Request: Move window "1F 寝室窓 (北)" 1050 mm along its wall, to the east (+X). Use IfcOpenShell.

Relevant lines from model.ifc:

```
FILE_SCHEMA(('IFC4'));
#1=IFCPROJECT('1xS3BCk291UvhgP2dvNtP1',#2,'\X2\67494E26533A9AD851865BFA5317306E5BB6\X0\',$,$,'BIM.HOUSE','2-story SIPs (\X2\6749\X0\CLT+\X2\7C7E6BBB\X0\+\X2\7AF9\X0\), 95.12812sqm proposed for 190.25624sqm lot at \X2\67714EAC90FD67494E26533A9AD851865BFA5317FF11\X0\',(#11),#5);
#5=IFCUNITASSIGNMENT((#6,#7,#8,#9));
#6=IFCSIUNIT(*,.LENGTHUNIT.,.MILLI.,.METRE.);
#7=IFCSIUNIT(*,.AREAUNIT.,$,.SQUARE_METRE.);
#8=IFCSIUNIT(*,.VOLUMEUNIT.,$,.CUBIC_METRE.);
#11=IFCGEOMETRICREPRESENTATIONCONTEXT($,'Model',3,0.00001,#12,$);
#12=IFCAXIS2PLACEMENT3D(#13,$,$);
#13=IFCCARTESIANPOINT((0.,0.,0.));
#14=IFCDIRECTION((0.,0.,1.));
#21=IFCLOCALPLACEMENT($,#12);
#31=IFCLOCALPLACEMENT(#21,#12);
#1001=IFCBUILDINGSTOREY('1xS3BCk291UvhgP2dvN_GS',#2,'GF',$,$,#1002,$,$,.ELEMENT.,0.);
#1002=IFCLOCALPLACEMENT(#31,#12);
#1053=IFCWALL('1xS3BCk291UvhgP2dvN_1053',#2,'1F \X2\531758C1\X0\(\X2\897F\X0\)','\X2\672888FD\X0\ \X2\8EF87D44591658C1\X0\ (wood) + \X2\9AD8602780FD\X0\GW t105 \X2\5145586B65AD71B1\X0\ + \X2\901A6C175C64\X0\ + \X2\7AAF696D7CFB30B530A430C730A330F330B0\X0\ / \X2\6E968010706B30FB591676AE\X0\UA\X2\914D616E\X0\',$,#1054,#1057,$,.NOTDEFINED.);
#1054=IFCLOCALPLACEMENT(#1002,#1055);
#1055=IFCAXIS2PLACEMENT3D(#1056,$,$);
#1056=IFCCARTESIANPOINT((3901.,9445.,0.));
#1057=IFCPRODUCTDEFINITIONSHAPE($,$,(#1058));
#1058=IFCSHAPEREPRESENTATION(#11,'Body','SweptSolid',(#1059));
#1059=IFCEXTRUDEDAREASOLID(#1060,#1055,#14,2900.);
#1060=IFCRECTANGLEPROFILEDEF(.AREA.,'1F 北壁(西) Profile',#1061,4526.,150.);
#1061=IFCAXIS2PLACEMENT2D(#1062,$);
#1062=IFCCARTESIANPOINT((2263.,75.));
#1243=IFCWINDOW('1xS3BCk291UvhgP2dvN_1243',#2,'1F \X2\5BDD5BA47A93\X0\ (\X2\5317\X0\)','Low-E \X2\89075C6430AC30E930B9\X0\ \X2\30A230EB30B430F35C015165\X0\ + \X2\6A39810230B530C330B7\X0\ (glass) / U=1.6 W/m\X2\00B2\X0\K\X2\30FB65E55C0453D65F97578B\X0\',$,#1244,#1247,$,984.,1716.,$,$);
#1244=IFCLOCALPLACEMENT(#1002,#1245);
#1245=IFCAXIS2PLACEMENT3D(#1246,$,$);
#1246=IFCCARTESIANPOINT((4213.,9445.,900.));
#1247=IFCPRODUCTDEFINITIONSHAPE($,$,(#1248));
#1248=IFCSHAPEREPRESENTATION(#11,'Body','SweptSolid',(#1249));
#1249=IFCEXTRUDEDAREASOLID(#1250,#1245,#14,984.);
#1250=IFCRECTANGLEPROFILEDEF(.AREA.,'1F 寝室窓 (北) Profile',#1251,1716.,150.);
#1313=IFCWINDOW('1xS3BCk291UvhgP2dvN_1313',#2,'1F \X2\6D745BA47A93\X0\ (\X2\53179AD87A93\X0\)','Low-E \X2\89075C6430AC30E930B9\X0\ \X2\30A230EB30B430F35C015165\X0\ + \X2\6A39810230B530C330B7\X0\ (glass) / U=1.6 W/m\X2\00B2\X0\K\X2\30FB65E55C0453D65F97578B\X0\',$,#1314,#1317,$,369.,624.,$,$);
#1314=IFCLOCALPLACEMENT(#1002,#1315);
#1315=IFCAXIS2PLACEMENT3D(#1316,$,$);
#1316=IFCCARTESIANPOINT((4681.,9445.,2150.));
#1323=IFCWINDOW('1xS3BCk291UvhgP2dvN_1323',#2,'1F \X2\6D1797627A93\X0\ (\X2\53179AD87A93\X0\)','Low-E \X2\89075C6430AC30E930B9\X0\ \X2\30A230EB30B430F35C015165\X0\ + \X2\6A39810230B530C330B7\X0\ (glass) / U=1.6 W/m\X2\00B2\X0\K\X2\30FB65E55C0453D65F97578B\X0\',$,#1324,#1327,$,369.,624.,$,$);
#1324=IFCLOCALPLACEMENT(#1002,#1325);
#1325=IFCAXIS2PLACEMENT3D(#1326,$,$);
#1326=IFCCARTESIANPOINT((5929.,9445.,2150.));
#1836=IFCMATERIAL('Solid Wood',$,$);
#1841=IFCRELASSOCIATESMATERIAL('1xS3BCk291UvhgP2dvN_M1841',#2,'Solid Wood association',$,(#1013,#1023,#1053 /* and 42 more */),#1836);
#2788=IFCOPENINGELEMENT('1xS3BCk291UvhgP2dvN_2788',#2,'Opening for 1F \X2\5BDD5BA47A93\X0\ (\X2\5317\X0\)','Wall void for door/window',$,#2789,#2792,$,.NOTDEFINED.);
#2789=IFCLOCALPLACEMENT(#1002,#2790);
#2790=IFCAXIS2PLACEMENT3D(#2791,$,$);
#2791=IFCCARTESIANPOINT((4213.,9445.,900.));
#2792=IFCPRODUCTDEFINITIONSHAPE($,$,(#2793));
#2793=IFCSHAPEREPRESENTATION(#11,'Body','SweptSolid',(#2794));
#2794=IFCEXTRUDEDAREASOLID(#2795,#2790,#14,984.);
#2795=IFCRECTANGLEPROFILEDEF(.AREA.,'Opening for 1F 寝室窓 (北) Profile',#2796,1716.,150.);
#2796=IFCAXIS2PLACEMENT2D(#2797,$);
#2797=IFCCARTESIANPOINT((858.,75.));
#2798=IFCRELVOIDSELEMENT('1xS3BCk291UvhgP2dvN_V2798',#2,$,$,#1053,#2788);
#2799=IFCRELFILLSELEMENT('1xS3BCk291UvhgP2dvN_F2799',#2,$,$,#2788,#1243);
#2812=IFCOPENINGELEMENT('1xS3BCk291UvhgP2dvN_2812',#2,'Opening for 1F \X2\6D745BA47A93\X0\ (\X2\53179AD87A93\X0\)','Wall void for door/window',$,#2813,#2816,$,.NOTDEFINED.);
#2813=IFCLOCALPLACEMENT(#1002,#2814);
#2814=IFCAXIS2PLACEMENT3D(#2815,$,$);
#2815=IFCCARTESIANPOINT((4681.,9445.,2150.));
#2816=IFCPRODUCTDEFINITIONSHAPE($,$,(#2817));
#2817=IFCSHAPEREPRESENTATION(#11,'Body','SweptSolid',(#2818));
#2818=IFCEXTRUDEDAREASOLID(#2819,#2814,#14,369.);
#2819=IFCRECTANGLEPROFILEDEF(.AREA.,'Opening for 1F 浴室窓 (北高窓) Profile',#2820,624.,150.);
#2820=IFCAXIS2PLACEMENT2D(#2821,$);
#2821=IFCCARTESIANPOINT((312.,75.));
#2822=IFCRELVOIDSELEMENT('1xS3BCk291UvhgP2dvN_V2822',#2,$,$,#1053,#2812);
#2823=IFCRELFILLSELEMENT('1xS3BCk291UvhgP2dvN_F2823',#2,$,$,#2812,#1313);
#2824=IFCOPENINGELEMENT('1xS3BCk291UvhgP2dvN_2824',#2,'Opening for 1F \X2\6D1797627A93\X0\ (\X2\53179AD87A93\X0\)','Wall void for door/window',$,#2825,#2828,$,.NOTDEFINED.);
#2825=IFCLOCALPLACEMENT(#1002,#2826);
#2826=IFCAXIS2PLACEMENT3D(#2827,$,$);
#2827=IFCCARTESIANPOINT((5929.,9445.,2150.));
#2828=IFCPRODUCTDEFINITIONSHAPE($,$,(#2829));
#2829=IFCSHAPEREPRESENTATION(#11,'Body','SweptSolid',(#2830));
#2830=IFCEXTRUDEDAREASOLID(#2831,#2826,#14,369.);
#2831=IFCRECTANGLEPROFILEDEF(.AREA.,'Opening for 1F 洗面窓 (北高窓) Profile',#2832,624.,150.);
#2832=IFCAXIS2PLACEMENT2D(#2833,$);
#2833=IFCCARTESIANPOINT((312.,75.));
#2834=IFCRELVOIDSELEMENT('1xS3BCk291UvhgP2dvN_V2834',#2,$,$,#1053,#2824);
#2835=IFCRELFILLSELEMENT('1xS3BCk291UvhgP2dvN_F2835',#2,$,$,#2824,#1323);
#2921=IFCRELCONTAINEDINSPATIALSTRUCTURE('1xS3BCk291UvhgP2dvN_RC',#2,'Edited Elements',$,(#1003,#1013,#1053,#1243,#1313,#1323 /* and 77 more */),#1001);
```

```python
import ifcopenshell
import ifcopenshell.api.geometry
import ifcopenshell.util.placement
import ifcopenshell.util.unit

model = ifcopenshell.open("model.ifc")
unit_scale = ifcopenshell.util.unit.calculate_unit_scale(model)

window = model.by_guid("1xS3BCk291UvhgP2dvN_1243")
opening = window.FillsVoids[0].RelatingOpeningElement
wall = opening.VoidsElements[0].RelatingBuildingElement

wall_matrix = ifcopenshell.util.placement.get_local_placement(wall.ObjectPlacement)
shift = wall_matrix[:3, 0] * 1.05 / unit_scale
before = ifcopenshell.util.placement.get_local_placement(window.ObjectPlacement)[:3, 3].copy()

# The window is not placed relative to its opening, so move both.
for product in (opening, window):
    matrix = ifcopenshell.util.placement.get_local_placement(product.ObjectPlacement)
    matrix[:3, 3] += shift
    ifcopenshell.api.geometry.edit_object_placement(model, product=product, matrix=matrix, is_si=False)

after = ifcopenshell.util.placement.get_local_placement(window.ObjectPlacement)[:3, 3]
print("window moved by", (after - before).round(3) + 0.0)

model.write("model_rev.ifc")
```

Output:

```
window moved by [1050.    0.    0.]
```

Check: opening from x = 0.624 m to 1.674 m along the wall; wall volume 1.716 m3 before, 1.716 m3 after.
